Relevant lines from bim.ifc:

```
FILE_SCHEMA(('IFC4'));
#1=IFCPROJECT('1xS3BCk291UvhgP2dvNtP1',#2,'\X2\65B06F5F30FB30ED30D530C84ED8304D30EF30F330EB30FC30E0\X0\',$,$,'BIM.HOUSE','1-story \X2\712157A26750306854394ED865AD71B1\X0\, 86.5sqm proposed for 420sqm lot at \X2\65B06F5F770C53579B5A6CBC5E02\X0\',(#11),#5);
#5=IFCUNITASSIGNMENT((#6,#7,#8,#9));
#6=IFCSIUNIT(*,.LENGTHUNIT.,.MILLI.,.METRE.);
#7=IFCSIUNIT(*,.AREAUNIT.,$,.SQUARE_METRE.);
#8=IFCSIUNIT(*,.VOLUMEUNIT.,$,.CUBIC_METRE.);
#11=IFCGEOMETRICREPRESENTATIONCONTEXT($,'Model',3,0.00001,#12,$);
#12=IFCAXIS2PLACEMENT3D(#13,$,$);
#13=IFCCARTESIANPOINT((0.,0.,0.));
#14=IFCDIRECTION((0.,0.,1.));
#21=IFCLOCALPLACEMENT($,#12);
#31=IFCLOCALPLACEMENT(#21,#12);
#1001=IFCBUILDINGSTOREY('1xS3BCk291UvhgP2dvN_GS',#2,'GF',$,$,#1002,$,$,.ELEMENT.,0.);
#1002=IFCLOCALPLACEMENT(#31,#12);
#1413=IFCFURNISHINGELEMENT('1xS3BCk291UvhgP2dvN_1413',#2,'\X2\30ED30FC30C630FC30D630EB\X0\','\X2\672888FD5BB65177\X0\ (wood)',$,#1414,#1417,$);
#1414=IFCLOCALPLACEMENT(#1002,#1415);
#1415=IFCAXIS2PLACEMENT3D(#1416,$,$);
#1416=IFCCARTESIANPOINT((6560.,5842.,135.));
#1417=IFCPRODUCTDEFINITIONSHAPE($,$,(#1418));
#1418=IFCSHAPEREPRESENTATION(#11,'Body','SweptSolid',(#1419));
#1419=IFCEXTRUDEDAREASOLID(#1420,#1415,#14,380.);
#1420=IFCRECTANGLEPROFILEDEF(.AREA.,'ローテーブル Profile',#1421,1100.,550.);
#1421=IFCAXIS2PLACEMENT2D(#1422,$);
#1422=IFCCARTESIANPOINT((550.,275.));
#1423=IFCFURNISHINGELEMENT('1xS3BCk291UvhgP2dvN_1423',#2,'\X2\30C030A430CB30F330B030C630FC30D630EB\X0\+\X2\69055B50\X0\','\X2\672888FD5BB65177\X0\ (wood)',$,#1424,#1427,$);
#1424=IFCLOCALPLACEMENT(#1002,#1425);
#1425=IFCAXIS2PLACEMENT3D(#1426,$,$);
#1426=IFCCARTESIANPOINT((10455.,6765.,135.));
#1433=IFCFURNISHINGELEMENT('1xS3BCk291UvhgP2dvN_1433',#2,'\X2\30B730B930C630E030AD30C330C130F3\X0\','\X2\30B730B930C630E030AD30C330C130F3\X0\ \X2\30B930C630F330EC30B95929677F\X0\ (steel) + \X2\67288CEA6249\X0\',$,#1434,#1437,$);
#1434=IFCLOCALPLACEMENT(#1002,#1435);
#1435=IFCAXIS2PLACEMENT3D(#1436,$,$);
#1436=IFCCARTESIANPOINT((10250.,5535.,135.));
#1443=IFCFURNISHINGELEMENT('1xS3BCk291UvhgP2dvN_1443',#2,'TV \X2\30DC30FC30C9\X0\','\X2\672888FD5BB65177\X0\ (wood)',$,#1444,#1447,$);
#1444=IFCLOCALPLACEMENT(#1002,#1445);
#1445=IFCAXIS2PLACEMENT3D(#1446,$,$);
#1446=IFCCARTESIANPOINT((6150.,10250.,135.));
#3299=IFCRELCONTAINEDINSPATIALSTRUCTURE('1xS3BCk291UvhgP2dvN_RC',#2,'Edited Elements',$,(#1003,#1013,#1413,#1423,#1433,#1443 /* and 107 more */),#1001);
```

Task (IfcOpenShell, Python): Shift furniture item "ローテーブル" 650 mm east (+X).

```python
import ifcopenshell
import ifcopenshell.api.geometry
import ifcopenshell.util.placement
import ifcopenshell.util.unit

model = ifcopenshell.open("bim.ifc")
unit_scale = ifcopenshell.util.unit.calculate_unit_scale(model)

item = model.by_guid("1xS3BCk291UvhgP2dvN_1413")
matrix = ifcopenshell.util.placement.get_local_placement(item.ObjectPlacement)
matrix[0, 3] += 0.65 / unit_scale
ifcopenshell.api.geometry.edit_object_placement(model, product=item, matrix=matrix, is_si=False)

print(ifcopenshell.util.placement.get_local_placement(item.ObjectPlacement).round(3) + 0.0)

model.write("bim_v2.ifc")
```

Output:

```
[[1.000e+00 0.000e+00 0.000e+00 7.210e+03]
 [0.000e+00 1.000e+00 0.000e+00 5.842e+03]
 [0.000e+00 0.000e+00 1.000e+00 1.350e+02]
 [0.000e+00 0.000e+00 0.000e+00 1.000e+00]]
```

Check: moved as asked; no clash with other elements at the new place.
